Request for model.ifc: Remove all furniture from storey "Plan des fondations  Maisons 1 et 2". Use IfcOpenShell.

First a look at what the model holds.

```python
import ifcopenshell
import ifcopenshell.util.element

model = ifcopenshell.open("model.ifc")
print(model.schema)
storey = next(s for s in model.by_type("IfcBuildingStorey") if s.Name == "Plan des fondations  Maisons 1 et 2")
furniture = [e for e in ifcopenshell.util.element.get_decomposition(storey) if e.is_a("IfcFurnishingElement")]
seen = {}
for e in furniture:
    element_type = ifcopenshell.util.element.get_type(e)
    name = element_type.Name if element_type not in (None, e) else None
    seen[name] = seen.get(name, 0) + 1
for name, count in sorted(seen.items(), key=str):
    print(count, "x", name)
```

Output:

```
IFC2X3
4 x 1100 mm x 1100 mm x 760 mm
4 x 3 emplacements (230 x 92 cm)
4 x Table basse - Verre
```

```python
import ifcopenshell
import ifcopenshell.api.root
import ifcopenshell.util.element

model = ifcopenshell.open("model.ifc")

storey = next(s for s in model.by_type("IfcBuildingStorey") if s.Name == "Plan des fondations  Maisons 1 et 2")
furniture = [e for e in ifcopenshell.util.element.get_decomposition(storey) if e.is_a("IfcFurnishingElement")]

for e in furniture:
    ifcopenshell.api.root.remove_product(model, product=e)
print(len(furniture), "removed")

model.write("model_updated.ifc")
```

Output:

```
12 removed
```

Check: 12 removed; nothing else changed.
